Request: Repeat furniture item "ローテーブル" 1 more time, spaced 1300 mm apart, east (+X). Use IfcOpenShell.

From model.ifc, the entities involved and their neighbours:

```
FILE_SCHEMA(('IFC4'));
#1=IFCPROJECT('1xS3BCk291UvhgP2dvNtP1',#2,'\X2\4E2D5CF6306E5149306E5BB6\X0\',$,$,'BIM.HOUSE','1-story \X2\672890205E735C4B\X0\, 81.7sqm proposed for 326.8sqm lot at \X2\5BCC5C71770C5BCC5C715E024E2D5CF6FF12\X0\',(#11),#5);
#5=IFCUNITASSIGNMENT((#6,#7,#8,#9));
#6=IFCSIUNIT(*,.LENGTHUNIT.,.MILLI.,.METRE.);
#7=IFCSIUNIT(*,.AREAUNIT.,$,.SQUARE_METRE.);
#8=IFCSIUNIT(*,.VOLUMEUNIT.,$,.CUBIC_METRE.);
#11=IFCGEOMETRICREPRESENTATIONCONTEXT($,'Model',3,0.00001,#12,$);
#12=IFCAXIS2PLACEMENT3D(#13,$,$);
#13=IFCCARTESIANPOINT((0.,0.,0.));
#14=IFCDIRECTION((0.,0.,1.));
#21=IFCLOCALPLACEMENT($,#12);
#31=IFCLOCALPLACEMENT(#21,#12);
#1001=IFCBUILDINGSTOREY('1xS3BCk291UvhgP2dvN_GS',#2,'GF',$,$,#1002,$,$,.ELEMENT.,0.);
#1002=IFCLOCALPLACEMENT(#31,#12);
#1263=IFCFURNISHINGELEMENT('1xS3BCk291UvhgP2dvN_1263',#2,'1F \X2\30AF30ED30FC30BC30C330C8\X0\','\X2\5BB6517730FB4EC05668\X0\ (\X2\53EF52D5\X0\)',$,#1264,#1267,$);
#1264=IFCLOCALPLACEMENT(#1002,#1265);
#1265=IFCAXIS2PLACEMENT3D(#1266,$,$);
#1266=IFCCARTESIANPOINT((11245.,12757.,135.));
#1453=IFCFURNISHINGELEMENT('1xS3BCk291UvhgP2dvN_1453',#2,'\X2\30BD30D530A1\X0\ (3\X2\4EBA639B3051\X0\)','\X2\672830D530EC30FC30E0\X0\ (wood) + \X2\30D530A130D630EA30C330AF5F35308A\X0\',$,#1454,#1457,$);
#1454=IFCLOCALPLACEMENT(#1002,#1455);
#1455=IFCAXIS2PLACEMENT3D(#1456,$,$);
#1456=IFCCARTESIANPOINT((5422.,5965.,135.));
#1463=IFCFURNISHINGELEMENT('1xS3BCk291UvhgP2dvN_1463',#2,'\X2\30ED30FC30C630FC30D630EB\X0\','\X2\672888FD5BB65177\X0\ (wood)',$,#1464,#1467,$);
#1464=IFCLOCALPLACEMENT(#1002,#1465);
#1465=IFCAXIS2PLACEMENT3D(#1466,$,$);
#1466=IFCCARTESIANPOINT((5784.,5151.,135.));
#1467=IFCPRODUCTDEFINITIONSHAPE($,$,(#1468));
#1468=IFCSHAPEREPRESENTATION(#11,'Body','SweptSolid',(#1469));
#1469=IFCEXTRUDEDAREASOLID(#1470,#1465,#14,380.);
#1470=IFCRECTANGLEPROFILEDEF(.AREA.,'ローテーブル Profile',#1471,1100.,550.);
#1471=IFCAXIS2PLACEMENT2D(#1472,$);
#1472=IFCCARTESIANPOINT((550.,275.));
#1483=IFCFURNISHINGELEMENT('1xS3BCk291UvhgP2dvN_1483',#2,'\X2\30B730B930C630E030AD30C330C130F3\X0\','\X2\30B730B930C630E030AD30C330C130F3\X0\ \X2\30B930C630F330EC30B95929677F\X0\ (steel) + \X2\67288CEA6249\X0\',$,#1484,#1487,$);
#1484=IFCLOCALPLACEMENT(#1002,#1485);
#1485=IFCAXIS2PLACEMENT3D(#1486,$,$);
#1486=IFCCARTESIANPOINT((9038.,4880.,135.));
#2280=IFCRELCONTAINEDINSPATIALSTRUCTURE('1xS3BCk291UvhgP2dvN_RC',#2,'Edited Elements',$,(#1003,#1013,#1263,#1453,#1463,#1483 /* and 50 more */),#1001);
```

```python
import numpy as np
import ifcopenshell
import ifcopenshell.api.geometry
import ifcopenshell.api.root
import ifcopenshell.util.element
import ifcopenshell.util.placement
import ifcopenshell.util.unit

model = ifcopenshell.open("model.ifc")
unit_scale = ifcopenshell.util.unit.calculate_unit_scale(model)


def reuse_history(source, copy):
    """copy_class also copies each property set's owner history, people and application; keep the originals."""
    for rel in copy.IsDefinedBy:
        if rel.is_a("IfcRelDefinesByProperties") and (history := rel.RelatingPropertyDefinition.OwnerHistory):
            rel.RelatingPropertyDefinition.OwnerHistory = source.OwnerHistory
            ifcopenshell.util.element.remove_deep2(model, history)


source = model.by_id(1463)
base = ifcopenshell.util.placement.get_local_placement(source.ObjectPlacement)
step = np.array([1.0, 0.0, 0.0]) * 1.3 / unit_scale

for i in range(1, 2):
    copy = ifcopenshell.api.root.copy_class(model, product=source)
    copy.Representation = ifcopenshell.util.element.copy_deep(
        model, source.Representation, exclude=["IfcGeometricRepresentationContext", "IfcRepresentationMap"]
    )
    reuse_history(source, copy)
    matrix = base.copy()
    matrix[:3, 3] += i * step
    print("added at", matrix[:3, 3].round(3) + 0.0)
    ifcopenshell.api.geometry.edit_object_placement(model, product=copy, matrix=matrix, is_si=False)

model.write("model-out.ifc")
```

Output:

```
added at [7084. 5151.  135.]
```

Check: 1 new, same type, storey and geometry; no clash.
